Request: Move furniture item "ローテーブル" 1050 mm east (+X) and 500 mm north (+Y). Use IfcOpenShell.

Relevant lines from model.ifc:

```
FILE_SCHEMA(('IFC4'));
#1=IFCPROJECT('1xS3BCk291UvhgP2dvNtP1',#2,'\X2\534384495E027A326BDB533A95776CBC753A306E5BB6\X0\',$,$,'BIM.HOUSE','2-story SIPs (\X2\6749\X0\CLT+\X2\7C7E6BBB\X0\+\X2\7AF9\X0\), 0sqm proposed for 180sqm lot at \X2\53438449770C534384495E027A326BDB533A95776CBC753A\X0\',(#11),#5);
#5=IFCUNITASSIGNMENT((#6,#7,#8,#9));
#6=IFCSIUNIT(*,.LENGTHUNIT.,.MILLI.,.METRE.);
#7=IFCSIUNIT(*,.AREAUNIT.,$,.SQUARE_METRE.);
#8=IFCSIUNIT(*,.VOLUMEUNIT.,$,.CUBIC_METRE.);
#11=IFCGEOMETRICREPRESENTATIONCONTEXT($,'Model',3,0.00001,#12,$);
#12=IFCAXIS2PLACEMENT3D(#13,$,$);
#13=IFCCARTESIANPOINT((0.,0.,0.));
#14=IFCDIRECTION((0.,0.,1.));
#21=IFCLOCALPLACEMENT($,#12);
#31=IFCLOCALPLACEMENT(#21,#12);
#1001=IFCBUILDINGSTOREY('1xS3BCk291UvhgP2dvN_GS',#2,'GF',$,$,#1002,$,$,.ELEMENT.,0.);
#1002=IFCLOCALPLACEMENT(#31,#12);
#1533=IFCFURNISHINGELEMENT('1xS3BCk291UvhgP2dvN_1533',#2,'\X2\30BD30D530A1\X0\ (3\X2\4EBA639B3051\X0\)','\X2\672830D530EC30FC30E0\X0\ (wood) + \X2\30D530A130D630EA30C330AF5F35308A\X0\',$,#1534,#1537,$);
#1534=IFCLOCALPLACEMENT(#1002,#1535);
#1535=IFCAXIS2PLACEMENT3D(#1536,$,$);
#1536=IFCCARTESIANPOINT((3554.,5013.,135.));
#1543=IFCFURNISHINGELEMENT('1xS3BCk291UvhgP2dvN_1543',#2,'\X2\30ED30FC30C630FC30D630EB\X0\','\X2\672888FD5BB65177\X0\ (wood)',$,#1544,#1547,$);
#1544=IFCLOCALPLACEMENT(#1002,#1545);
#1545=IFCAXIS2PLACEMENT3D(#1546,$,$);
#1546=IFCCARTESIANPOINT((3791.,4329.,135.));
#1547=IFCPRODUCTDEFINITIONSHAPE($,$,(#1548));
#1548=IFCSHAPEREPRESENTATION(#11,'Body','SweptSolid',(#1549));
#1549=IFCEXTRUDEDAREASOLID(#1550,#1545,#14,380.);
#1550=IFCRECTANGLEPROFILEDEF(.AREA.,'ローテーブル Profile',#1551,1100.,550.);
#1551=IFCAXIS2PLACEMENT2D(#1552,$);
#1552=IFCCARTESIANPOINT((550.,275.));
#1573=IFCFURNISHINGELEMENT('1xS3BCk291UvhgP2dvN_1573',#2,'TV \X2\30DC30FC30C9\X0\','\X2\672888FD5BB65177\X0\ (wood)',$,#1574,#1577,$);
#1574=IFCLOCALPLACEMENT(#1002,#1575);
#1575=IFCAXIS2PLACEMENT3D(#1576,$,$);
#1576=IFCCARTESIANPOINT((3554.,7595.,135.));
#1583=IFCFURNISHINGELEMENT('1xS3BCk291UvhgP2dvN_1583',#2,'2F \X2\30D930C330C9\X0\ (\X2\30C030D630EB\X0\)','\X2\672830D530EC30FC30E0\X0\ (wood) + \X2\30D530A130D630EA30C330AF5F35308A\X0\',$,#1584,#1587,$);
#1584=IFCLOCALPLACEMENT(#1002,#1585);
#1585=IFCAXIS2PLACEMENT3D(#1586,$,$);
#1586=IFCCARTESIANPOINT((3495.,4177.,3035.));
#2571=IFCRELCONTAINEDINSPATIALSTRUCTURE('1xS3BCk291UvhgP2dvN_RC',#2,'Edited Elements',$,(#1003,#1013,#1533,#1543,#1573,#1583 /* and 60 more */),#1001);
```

```python
import ifcopenshell
import ifcopenshell.api.geometry
import ifcopenshell.util.placement

model = ifcopenshell.open("model.ifc")

item = model.by_id(1543)
matrix = ifcopenshell.util.placement.get_local_placement(item.ObjectPlacement)
matrix[0, 3] += 1050.0
matrix[1, 3] += 500.0
ifcopenshell.api.geometry.edit_object_placement(model, product=item, matrix=matrix, is_si=False)

print(ifcopenshell.util.placement.get_local_placement(item.ObjectPlacement).round(3) + 0.0)

model.write("model_edited.ifc")
```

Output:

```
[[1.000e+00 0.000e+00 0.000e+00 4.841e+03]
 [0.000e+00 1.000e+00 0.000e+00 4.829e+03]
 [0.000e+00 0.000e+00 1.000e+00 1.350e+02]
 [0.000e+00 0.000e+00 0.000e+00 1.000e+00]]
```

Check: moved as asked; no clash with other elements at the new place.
